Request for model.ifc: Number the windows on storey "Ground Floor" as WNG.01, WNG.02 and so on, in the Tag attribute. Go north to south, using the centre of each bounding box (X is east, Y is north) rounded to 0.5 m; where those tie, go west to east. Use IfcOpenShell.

First a look at what the model holds.

```python
import ifcopenshell
import ifcopenshell.util.element
import ifcopenshell.util.placement

model = ifcopenshell.open("model.ifc")
print(model.schema)
storey = next(s for s in model.by_type("IfcBuildingStorey") if s.Name == "Ground Floor")
windows = [e for e in ifcopenshell.util.element.get_decomposition(storey) if e.is_a("IfcWindow")]
for e in sorted(windows, key=lambda e: e.id()):
    origin = ifcopenshell.util.placement.get_local_placement(e.ObjectPlacement)[:3, 3]
    print(e.id(), e.Tag, e.Name, origin.round(2) + 0.0, sep=" | ")
```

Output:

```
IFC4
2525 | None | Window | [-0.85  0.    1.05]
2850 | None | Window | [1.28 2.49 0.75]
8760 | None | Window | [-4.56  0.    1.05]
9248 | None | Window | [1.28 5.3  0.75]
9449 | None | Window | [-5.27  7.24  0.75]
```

```python
import ifcopenshell
import ifcopenshell.geom
import ifcopenshell.util.element
import ifcopenshell.util.shape

model = ifcopenshell.open("model.ifc")
settings = ifcopenshell.geom.settings()
settings.set("use-world-coords", True)


def centre(element):
    shape = ifcopenshell.geom.create_shape(settings, element)
    return ifcopenshell.util.shape.get_bbox_centroid(shape.geometry)


storey = next(s for s in model.by_type("IfcBuildingStorey") if s.Name == "Ground Floor")
windows = [e for e in ifcopenshell.util.element.get_decomposition(storey) if e.is_a("IfcWindow")]

# Insertion points can sit at a corner or the storey origin, so sort by the geometry (in metres).
centres = {e: centre(e) for e in windows}
windows.sort(key=lambda e: (-round(centres[e][1] / 0.5), centres[e][0]))

for i, e in enumerate(windows, start=1):
    number = f"WNG.{i:02d}"
    e.Tag = number
    print(e.id(), number)

model.write("model_v2.ifc")
```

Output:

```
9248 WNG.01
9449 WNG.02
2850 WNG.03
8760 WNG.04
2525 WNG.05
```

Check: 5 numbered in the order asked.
